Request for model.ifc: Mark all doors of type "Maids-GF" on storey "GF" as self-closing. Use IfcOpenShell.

First a look at what the model holds.

```python
import ifcopenshell
import ifcopenshell.util.element

model = ifcopenshell.open("model.ifc")
print(model.schema)
storey = next(s for s in model.by_type("IfcBuildingStorey") if s.Name == "GF")
doors = [e for e in ifcopenshell.util.element.get_decomposition(storey) if e.is_a("IfcDoor")]
seen = {}
for e in doors:
    element_type = ifcopenshell.util.element.get_type(e)
    key = (element_type.Name if element_type != e and element_type else None, ifcopenshell.util.element.get_pset(e, "Pset_DoorCommon", "SelfClosing"))
    seen[key] = seen.get(key, 0) + 1
for (name, value), count in sorted(seen.items(), key=str):
    print(count, "x", name, "|", value)
```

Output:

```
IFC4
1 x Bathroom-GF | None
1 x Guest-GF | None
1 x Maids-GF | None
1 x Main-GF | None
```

```python
import ifcopenshell
import ifcopenshell.api.pset
import ifcopenshell.util.element

model = ifcopenshell.open("model.ifc")

storey = next(s for s in model.by_type("IfcBuildingStorey") if s.Name == "GF")
doors = [e for e in ifcopenshell.util.element.get_decomposition(storey) if e.is_a("IfcDoor")]

count = 0
for e in doors:
    element_type = ifcopenshell.util.element.get_type(e)
    if element_type in (None, e) or element_type.Name != "Maids-GF":
        continue
    # add_pset returns the element's existing set when there is one.
    pset = ifcopenshell.api.pset.add_pset(model, product=e, name="Pset_DoorCommon")
    ifcopenshell.api.pset.edit_pset(model, pset=pset, properties={"SelfClosing": True})
    count += 1

print(count, "doors updated")

model.write("model-out.ifc")
```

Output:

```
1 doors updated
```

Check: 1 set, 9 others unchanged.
